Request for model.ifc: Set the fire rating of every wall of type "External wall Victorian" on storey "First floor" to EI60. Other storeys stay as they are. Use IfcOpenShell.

First a look at what the model holds.

```python
import ifcopenshell
import ifcopenshell.util.element

model = ifcopenshell.open("model.ifc")
print(model.schema)
storey = next(s for s in model.by_type("IfcBuildingStorey") if s.Name == "First floor")
walls = [e for e in ifcopenshell.util.element.get_decomposition(storey) if e.is_a("IfcWall")]
seen = {}
for e in walls:
    element_type = ifcopenshell.util.element.get_type(e)
    key = (element_type.Name if element_type != e and element_type else None, ifcopenshell.util.element.get_pset(e, "Pset_WallCommon", "FireRating"))
    seen[key] = seen.get(key, 0) + 1
for (name, value), count in sorted(seen.items(), key=str):
    print(count, "x", name, "|", value)
```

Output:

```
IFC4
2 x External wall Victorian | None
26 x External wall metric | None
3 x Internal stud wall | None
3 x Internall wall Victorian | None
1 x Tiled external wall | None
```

```python
import ifcopenshell
import ifcopenshell.api.pset
import ifcopenshell.util.element

model = ifcopenshell.open("model.ifc")

storey = next(s for s in model.by_type("IfcBuildingStorey") if s.Name == "First floor")
walls = [e for e in ifcopenshell.util.element.get_decomposition(storey) if e.is_a("IfcWall")]

count = 0
for e in walls:
    element_type = ifcopenshell.util.element.get_type(e)
    if element_type in (None, e) or element_type.Name != "External wall Victorian":
        continue
    # add_pset returns the element's existing set when there is one.
    pset = ifcopenshell.api.pset.add_pset(model, product=e, name="Pset_WallCommon")
    ifcopenshell.api.pset.edit_pset(model, pset=pset, properties={"FireRating": "EI60"})
    count += 1

print(count, "walls updated")

model.write("model_rev.ifc")
```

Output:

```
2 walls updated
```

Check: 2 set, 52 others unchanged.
